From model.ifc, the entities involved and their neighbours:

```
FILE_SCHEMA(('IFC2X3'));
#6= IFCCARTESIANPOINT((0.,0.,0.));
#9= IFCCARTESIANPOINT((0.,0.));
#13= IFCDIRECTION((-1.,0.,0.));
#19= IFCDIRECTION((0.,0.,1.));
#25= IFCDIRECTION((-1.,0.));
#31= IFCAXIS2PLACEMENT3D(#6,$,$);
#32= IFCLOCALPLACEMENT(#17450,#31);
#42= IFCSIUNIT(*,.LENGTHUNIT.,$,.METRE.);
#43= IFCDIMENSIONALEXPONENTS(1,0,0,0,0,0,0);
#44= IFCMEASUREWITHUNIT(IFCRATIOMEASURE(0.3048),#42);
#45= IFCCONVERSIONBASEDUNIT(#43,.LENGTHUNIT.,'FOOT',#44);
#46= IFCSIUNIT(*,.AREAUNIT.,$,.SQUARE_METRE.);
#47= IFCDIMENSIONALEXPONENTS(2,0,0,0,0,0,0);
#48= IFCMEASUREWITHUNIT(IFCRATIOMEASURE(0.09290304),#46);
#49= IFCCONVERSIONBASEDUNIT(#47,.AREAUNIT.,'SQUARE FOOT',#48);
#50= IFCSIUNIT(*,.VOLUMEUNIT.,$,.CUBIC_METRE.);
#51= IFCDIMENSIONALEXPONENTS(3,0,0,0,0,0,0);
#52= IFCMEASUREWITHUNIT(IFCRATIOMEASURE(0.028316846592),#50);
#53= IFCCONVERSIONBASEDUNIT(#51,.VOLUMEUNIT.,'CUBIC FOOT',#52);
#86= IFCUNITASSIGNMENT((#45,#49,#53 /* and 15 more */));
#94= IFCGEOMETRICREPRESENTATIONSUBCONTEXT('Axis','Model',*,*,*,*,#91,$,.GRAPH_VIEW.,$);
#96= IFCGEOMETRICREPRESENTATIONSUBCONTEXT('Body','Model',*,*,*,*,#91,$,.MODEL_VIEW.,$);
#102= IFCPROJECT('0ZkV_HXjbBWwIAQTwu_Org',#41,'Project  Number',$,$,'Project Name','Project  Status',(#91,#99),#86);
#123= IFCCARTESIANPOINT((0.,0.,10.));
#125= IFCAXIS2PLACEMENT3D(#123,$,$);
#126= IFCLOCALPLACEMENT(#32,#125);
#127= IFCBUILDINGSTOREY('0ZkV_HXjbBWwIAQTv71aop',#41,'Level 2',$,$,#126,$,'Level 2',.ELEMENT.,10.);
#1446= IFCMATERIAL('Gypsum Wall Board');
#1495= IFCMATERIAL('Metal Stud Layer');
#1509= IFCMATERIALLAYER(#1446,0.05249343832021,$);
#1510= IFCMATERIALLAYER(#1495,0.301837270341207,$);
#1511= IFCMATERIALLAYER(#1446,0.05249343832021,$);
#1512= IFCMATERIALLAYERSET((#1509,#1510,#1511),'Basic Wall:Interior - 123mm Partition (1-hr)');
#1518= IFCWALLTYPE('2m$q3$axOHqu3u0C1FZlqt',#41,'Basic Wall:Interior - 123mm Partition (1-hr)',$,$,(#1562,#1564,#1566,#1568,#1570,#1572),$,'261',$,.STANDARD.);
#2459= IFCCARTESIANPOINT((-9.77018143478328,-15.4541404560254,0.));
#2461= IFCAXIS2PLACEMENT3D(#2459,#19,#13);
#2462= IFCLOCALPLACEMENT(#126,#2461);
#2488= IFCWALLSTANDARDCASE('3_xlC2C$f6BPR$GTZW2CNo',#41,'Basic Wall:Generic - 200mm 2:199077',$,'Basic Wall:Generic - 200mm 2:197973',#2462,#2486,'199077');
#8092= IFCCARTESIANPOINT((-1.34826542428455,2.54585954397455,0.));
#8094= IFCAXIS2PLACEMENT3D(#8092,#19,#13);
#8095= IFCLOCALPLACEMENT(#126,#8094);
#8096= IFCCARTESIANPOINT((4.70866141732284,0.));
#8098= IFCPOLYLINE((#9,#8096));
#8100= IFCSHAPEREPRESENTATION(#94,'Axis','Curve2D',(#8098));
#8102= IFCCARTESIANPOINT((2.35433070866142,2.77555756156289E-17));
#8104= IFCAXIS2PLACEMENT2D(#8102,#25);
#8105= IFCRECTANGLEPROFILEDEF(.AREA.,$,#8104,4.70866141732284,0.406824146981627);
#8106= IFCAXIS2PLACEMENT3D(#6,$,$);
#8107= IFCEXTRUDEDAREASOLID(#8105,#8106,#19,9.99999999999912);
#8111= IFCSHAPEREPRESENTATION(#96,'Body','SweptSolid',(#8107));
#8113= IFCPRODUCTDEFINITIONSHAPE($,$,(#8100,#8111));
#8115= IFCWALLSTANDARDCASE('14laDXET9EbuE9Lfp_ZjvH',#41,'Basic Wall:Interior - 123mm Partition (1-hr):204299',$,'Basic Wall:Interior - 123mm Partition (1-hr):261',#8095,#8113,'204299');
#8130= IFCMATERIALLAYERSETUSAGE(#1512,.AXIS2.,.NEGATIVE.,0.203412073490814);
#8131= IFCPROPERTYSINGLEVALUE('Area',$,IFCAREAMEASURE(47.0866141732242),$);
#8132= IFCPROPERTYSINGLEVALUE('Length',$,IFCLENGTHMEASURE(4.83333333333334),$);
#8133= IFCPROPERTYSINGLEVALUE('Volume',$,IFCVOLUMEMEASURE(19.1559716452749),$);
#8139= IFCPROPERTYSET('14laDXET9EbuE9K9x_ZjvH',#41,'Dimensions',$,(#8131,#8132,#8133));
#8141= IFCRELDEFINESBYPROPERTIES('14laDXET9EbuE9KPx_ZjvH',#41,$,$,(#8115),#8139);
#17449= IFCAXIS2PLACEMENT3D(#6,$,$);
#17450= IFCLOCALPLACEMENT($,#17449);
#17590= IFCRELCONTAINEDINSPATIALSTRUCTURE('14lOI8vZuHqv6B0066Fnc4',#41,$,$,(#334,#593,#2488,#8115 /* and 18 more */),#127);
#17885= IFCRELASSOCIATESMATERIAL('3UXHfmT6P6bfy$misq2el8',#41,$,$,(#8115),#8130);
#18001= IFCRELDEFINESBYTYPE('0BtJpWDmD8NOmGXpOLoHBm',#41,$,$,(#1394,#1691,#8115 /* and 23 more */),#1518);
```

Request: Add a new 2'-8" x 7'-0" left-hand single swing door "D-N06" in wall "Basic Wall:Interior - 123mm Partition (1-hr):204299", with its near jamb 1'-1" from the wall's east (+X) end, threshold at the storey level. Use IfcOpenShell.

```python
import numpy as np
import ifcopenshell
import ifcopenshell.api.feature
import ifcopenshell.api.geometry
import ifcopenshell.api.pset
import ifcopenshell.api.root
import ifcopenshell.api.spatial
import ifcopenshell.api.type
import ifcopenshell.geom
import ifcopenshell.util.element
import ifcopenshell.util.placement
import ifcopenshell.util.representation
import ifcopenshell.util.shape
import ifcopenshell.util.unit

model = ifcopenshell.open("model.ifc")
unit_scale = ifcopenshell.util.unit.calculate_unit_scale(model)
area_scale = ifcopenshell.util.unit.calculate_unit_scale(model, "AREAUNIT")
volume_scale = ifcopenshell.util.unit.calculate_unit_scale(model, "VOLUMEUNIT")
settings = ifcopenshell.geom.settings()


def volume(element):
    """Net volume in cubic metres, openings subtracted."""
    shape = ifcopenshell.geom.create_shape(settings, element)
    return ifcopenshell.util.shape.get_volume(shape.geometry)


wall = model.by_guid("14laDXET9EbuE9Lfp_ZjvH")
storey = ifcopenshell.util.element.get_container(wall, ifc_class="IfcBuildingStorey")
context = ifcopenshell.util.representation.get_context(model, "Model", "Body", "MODEL_VIEW")
before = volume(wall)

width, height, from_end, sill = 0.8128, 2.1336, 0.3302, 0.0  # metres

# The wall runs along its own X axis, and the end named is its -X end.
wall_shape = ifcopenshell.geom.create_shape(settings, wall)
x, y, z = ifcopenshell.util.shape.get_vertices(wall_shape.geometry).T
start = x.min() + from_end
face, thickness = float(y.min()), float(y.max() - y.min())
wall_matrix = ifcopenshell.util.placement.get_local_placement(wall.ObjectPlacement)
level = ifcopenshell.util.placement.get_local_placement(storey.ObjectPlacement)[2, 3]


def in_wall(x, y):
    """Placement at x, y metres in the wall's axes, at sill height."""
    matrix = wall_matrix.copy()
    matrix[:, 3] = wall_matrix @ np.array([x / unit_scale, y / unit_scale, 0.0, 1.0])
    matrix[2, 3] = level + sill / unit_scale
    return matrix


# Opening: a box that overshoots both wall faces by 50 mm.
opening = ifcopenshell.api.root.create_entity(model, ifc_class="IfcOpeningElement")
box = ifcopenshell.api.geometry.add_wall_representation(
    model, context=context, length=width, height=height, thickness=thickness + 0.1
)
ifcopenshell.api.geometry.assign_representation(model, product=opening, representation=box)
ifcopenshell.api.geometry.edit_object_placement(model, product=opening, matrix=in_wall(start, face - 0.05), is_si=False)
ifcopenshell.api.feature.add_feature(model, feature=opening, element=wall)

door = ifcopenshell.api.root.create_entity(model, ifc_class="IfcDoor", name="D-N06")
door.OverallWidth, door.OverallHeight = width / unit_scale, height / unit_scale
body = ifcopenshell.api.geometry.add_door_representation(
    model,
    context=context,
    overall_width=door.OverallWidth,
    overall_height=door.OverallHeight,
    operation_type="SINGLE_SWING_LEFT",
    lining_properties={"LiningDepth": thickness / unit_scale, "ThresholdDepth": thickness / unit_scale},
)
ifcopenshell.api.geometry.assign_representation(model, product=door, representation=body)
ifcopenshell.api.spatial.assign_container(model, products=[door], relating_structure=storey)
fills = ifcopenshell.api.feature.add_filling(model, opening=opening, element=door)
fills.OwnerHistory = door.OwnerHistory  # required in IFC2X3

# IFC2X3 keeps the operation on the door style.
style = ifcopenshell.api.root.create_entity(model, ifc_class="IfcDoorStyle", name="D-N06")
style.OperationType, style.ConstructionType = "SINGLE_SWING_LEFT", "NOTDEFINED"
style.ParameterTakesPrecedence = style.Sizeable = False
ifcopenshell.api.type.assign_type(model, related_objects=[door], relating_type=style)

# The lining spans the wall, so the door starts at the wall face.
ifcopenshell.api.geometry.edit_object_placement(model, product=door, matrix=in_wall(start, face), is_si=False)

after = volume(wall)

# Update the wall's stored quantities.
pset = model.by_id(ifcopenshell.util.element.get_pset(wall, "Dimensions", should_inherit=False)["id"])
ifcopenshell.api.pset.edit_pset(model, pset=pset, properties={
    "Area": model.create_entity("IfcAreaMeasure", after / thickness / area_scale),
    "Volume": model.create_entity("IfcVolumeMeasure", after / volume_scale),
})

print(f"wall volume {before:.3f} -> {after:.3f} m3")

model.write("model-out.ifc")
```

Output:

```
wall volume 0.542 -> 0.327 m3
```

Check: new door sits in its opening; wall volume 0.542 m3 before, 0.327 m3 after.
